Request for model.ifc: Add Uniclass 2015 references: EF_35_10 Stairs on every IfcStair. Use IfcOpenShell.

First a look at what the model holds.

```python
import ifcopenshell

model = ifcopenshell.open("model.ifc")
print(model.schema)
print("classifications:", [c.Name for c in model.by_type("IfcClassification")])
for ifc_class in ("IfcDoor", "IfcRoof", "IfcStair", "IfcWall", "IfcWindow"):
    print(ifc_class, len(model.by_type(ifc_class)))
```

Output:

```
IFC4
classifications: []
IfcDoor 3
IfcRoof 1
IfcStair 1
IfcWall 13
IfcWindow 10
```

```python
import ifcopenshell
import ifcopenshell.api.classification

model = ifcopenshell.open("model.ifc")

system = ifcopenshell.api.classification.add_classification(model, classification="Uniclass 2015")

codes = {
    "IfcStair": ("EF_35_10", "Stairs"),
}
for ifc_class, (code, name) in codes.items():
    products = model.by_type(ifc_class)
    ifcopenshell.api.classification.add_reference(
        model, products=products, classification=system, identification=code, name=name
    )
    print(code, len(products))

model.write("model_v2.ifc")
```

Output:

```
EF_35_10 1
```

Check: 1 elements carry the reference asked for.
